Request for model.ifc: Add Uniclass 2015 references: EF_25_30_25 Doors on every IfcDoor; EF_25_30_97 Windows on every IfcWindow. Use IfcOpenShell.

First a look at what the model holds.

```python
import ifcopenshell

model = ifcopenshell.open("model.ifc")
print(model.schema)
print("classifications:", [c.Name for c in model.by_type("IfcClassification")])
for ifc_class in ("IfcDoor", "IfcRoof", "IfcStair", "IfcWall", "IfcWindow"):
    print(ifc_class, len(model.by_type(ifc_class)))
```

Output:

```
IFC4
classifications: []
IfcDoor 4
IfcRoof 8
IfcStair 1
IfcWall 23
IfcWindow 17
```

```python
import ifcopenshell
import ifcopenshell.api.classification

model = ifcopenshell.open("model.ifc")

system = ifcopenshell.api.classification.add_classification(model, classification="Uniclass 2015")

codes = {
    "IfcDoor": ("EF_25_30_25", "Doors"),
    "IfcWindow": ("EF_25_30_97", "Windows"),
}
for ifc_class, (code, name) in codes.items():
    products = model.by_type(ifc_class)
    ifcopenshell.api.classification.add_reference(
        model, products=products, classification=system, identification=code, name=name
    )
    print(code, len(products))

model.write("model_updated.ifc")
```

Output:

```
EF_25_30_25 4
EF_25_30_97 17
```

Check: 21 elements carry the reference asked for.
